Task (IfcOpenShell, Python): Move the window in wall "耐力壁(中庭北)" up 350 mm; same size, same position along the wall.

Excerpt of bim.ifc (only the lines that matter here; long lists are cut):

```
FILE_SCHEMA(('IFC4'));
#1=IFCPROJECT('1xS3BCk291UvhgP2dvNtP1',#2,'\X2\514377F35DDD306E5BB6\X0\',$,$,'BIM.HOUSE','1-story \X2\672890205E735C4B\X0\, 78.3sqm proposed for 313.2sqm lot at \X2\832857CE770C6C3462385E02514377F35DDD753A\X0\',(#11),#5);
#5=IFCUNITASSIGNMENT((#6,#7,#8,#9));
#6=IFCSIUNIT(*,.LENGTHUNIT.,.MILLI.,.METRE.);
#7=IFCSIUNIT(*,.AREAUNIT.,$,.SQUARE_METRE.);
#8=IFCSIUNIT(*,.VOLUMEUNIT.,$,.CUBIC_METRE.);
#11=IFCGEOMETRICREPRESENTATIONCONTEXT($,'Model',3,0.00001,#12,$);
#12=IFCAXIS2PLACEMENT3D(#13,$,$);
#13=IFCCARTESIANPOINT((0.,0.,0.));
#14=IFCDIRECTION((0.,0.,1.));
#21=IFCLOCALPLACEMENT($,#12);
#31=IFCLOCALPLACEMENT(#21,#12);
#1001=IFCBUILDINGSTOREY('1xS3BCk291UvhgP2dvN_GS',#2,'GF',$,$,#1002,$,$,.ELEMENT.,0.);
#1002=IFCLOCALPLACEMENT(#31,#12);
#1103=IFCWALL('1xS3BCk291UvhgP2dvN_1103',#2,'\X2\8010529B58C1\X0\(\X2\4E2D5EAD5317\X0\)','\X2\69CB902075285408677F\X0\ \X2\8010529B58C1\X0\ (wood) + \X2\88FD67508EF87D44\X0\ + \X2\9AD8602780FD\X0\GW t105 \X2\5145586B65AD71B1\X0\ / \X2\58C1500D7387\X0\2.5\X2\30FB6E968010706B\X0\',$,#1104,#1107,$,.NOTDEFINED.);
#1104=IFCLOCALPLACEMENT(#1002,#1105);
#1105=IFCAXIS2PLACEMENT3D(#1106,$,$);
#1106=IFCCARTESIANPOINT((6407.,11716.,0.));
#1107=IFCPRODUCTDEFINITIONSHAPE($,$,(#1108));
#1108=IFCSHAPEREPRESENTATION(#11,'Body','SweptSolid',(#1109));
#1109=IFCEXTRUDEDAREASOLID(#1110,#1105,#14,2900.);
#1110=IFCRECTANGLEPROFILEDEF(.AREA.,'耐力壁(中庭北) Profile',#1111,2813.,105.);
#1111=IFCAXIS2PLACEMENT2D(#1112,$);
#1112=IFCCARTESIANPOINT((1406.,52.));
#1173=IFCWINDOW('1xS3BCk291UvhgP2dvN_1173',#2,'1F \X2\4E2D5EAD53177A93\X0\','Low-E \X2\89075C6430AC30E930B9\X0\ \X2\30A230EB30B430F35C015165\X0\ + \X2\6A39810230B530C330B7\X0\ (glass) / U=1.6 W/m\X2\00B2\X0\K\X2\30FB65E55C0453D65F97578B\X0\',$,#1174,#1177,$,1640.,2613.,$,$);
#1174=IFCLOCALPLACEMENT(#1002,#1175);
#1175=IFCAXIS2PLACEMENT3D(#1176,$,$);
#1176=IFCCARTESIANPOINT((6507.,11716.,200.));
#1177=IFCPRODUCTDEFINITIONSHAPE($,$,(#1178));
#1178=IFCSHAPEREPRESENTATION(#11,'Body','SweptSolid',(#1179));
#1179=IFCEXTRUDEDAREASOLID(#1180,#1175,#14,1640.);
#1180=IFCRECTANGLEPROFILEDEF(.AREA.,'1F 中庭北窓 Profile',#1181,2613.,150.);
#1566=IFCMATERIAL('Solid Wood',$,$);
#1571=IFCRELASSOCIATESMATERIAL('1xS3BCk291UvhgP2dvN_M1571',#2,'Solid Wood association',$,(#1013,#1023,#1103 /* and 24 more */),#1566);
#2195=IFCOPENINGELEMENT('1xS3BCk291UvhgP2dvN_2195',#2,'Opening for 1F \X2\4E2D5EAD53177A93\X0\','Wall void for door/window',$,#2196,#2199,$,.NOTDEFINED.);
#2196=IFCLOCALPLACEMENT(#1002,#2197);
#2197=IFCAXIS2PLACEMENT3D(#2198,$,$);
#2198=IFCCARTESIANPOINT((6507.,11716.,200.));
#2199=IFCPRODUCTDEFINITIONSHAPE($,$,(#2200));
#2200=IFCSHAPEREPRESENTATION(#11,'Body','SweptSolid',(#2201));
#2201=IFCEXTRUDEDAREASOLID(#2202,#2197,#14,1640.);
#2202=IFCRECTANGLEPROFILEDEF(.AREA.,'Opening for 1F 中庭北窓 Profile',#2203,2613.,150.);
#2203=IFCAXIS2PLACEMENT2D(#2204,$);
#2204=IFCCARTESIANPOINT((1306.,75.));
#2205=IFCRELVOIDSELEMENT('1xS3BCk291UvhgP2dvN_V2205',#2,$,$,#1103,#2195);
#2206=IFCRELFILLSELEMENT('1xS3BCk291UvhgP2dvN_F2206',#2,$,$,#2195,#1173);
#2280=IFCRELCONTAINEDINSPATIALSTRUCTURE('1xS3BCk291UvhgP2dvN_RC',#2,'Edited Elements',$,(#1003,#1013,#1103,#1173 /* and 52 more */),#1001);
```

```python
import numpy as np
import ifcopenshell
import ifcopenshell.api.geometry
import ifcopenshell.util.placement
import ifcopenshell.util.unit

model = ifcopenshell.open("bim.ifc")
unit_scale = ifcopenshell.util.unit.calculate_unit_scale(model)

window = model.by_guid("1xS3BCk291UvhgP2dvN_1173")
opening = window.FillsVoids[0].RelatingOpeningElement
dz = 0.35 / unit_scale

shift = np.array([0.0, 0.0, dz])
# The window is not placed relative to its opening, so move both.
for product in (opening, window):
    matrix = ifcopenshell.util.placement.get_local_placement(product.ObjectPlacement)
    matrix[:3, 3] += shift
    ifcopenshell.api.geometry.edit_object_placement(model, product=product, matrix=matrix, is_si=False)

print(f"moved by {dz * unit_scale:+.3f} m")

model.write("bim-out.ifc")
```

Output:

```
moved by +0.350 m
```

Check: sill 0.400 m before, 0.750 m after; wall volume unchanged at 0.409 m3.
